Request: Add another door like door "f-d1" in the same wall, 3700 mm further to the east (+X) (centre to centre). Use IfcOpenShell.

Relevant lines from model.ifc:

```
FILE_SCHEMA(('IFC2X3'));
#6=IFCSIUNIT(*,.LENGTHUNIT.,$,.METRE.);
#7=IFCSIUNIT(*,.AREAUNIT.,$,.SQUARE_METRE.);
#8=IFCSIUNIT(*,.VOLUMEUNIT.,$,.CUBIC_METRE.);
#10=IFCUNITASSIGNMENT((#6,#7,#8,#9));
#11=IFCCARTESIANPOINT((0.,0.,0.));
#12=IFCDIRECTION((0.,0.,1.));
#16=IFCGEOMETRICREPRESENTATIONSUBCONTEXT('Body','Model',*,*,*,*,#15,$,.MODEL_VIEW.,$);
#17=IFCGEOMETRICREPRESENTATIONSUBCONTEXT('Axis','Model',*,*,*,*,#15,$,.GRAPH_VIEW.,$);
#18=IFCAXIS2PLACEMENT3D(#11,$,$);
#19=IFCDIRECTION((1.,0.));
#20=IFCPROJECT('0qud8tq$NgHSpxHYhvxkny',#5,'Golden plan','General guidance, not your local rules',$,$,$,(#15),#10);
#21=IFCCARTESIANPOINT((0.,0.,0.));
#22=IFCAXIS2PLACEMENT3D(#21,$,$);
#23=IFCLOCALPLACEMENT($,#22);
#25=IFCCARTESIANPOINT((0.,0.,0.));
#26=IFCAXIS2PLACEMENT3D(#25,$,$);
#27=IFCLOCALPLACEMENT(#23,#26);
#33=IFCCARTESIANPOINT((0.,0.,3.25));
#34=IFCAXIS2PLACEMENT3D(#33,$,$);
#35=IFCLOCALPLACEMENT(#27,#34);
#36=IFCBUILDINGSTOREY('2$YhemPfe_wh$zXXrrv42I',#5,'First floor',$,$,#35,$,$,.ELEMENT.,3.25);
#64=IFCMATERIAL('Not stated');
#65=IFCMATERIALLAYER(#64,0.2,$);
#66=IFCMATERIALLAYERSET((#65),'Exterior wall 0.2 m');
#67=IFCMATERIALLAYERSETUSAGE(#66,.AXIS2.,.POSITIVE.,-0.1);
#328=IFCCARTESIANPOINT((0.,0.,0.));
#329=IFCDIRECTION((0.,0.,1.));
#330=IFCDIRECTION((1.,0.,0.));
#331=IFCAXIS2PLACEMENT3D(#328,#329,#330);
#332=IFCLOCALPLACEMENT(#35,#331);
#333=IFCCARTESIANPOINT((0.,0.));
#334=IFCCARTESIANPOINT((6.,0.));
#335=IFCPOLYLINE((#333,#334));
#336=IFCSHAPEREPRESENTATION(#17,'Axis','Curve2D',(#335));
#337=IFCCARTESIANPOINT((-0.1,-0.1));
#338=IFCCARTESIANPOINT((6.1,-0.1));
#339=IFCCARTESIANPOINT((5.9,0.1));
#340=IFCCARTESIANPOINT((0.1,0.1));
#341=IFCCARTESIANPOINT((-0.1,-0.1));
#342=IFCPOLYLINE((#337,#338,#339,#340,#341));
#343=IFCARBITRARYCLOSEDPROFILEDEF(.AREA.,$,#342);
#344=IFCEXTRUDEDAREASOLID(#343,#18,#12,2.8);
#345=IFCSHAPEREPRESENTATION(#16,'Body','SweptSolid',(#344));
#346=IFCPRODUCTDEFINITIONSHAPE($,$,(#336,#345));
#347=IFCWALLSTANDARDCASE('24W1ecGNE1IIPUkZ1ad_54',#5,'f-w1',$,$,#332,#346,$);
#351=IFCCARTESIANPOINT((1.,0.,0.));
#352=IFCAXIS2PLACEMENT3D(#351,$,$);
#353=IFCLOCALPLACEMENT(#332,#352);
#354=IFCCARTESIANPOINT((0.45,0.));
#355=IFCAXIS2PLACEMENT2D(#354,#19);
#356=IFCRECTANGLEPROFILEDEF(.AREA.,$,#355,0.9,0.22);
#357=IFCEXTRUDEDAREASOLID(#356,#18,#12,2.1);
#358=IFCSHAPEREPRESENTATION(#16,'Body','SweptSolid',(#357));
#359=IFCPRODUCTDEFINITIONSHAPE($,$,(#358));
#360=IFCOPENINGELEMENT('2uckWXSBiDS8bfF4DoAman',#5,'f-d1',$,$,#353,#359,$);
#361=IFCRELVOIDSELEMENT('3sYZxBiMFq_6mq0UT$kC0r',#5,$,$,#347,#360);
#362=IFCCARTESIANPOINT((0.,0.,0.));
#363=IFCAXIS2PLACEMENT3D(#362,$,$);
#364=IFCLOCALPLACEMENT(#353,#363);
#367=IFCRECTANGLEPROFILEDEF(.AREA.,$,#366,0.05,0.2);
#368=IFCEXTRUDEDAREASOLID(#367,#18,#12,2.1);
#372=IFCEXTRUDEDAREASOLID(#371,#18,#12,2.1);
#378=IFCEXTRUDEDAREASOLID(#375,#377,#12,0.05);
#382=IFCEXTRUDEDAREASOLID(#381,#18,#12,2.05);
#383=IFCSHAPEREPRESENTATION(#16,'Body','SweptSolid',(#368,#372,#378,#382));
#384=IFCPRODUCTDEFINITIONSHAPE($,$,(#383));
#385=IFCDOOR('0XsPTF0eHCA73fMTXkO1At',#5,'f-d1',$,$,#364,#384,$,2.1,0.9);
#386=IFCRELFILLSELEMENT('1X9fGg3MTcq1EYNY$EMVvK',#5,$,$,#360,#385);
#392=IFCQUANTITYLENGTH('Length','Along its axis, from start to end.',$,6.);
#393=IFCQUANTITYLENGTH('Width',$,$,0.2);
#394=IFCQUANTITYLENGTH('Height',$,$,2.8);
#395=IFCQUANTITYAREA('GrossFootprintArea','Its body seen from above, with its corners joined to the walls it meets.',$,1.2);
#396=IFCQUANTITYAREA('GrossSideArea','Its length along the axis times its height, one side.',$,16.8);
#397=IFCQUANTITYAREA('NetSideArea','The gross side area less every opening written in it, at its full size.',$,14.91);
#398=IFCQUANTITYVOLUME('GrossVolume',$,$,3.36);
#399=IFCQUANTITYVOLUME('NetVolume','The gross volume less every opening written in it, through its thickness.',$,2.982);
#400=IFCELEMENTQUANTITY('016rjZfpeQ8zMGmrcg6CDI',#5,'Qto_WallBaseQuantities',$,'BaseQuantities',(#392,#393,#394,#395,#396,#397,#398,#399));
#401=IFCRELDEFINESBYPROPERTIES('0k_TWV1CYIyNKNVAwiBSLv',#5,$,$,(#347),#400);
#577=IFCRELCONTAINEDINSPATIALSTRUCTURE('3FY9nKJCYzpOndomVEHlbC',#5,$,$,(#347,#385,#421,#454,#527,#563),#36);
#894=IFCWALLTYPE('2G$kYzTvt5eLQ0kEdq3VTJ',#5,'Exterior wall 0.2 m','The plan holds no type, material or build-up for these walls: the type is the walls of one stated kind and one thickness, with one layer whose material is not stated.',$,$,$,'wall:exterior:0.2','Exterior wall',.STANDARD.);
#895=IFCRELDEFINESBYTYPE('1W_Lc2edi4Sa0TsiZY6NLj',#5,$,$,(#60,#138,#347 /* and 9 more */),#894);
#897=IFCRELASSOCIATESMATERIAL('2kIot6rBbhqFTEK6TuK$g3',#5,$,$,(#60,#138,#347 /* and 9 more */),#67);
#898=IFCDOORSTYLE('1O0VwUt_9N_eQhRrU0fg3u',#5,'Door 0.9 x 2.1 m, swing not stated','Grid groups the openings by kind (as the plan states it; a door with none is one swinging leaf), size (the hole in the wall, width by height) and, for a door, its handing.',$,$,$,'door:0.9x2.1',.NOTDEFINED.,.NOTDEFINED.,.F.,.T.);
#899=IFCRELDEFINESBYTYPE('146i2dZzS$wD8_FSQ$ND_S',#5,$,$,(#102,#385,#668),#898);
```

```python
import ifcopenshell
import ifcopenshell.api.feature
import ifcopenshell.api.geometry
import ifcopenshell.api.pset
import ifcopenshell.api.root
import ifcopenshell.geom
import ifcopenshell.util.element
import ifcopenshell.util.placement
import ifcopenshell.util.shape
import ifcopenshell.util.unit

model = ifcopenshell.open("model.ifc")
unit_scale = ifcopenshell.util.unit.calculate_unit_scale(model)
area_scale = ifcopenshell.util.unit.calculate_unit_scale(model, "AREAUNIT")
volume_scale = ifcopenshell.util.unit.calculate_unit_scale(model, "VOLUMEUNIT")
settings = ifcopenshell.geom.settings()


def volume(element):
    """Net volume in cubic metres, openings subtracted."""
    shape = ifcopenshell.geom.create_shape(settings, element)
    return ifcopenshell.util.shape.get_volume(shape.geometry)


def reuse_history(source, copy):
    """copy_class also copies each property set's owner history, people and application; keep the originals."""
    for rel in copy.IsDefinedBy:
        if rel.is_a("IfcRelDefinesByProperties") and (history := rel.RelatingPropertyDefinition.OwnerHistory):
            rel.RelatingPropertyDefinition.OwnerHistory = source.OwnerHistory
            ifcopenshell.util.element.remove_deep2(model, history)


door = model.by_id(385)
opening = door.FillsVoids[0].RelatingOpeningElement
wall = opening.VoidsElements[0].RelatingBuildingElement
before = volume(wall)
shift = ifcopenshell.util.placement.get_local_placement(wall.ObjectPlacement)[:3, 0] * 3.7 / unit_scale

# copy_class copies the void relationship, type, container and properties, but no geometry.
new_opening = ifcopenshell.api.root.copy_class(model, product=opening)
new_opening.Representation = ifcopenshell.util.element.copy_deep(
    model, opening.Representation, exclude=["IfcGeometricRepresentationContext", "IfcRepresentationMap"]
)
new_door = ifcopenshell.api.root.copy_class(model, product=door)
new_door.Representation = ifcopenshell.util.element.copy_deep(
    model, door.Representation, exclude=["IfcGeometricRepresentationContext", "IfcRepresentationMap"]
)
reuse_history(door, new_door)
fills = ifcopenshell.api.feature.add_filling(model, opening=new_opening, element=new_door)
fills.OwnerHistory = new_door.OwnerHistory  # required in IFC2X3

for old, new in ((opening, new_opening), (door, new_door)):
    matrix = ifcopenshell.util.placement.get_local_placement(old.ObjectPlacement)
    matrix[:3, 3] += shift
    ifcopenshell.api.geometry.edit_object_placement(model, product=new, matrix=matrix, is_si=False)

after = volume(wall)
thickness = 0.2  # wall thickness in metres

# Update the wall's stored quantities.
qto = model.by_id(ifcopenshell.util.element.get_pset(wall, "Qto_WallBaseQuantities", should_inherit=False)["id"])
ifcopenshell.api.pset.edit_qto(model, qto=qto, properties={
    "NetSideArea": after / thickness / area_scale,
    "NetVolume": after / volume_scale,
})

print(f"wall volume {before:.3f} -> {after:.3f} m3")

model.write("model-out.ifc")
```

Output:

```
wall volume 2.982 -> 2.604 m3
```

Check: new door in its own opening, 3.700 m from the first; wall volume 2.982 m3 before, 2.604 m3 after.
